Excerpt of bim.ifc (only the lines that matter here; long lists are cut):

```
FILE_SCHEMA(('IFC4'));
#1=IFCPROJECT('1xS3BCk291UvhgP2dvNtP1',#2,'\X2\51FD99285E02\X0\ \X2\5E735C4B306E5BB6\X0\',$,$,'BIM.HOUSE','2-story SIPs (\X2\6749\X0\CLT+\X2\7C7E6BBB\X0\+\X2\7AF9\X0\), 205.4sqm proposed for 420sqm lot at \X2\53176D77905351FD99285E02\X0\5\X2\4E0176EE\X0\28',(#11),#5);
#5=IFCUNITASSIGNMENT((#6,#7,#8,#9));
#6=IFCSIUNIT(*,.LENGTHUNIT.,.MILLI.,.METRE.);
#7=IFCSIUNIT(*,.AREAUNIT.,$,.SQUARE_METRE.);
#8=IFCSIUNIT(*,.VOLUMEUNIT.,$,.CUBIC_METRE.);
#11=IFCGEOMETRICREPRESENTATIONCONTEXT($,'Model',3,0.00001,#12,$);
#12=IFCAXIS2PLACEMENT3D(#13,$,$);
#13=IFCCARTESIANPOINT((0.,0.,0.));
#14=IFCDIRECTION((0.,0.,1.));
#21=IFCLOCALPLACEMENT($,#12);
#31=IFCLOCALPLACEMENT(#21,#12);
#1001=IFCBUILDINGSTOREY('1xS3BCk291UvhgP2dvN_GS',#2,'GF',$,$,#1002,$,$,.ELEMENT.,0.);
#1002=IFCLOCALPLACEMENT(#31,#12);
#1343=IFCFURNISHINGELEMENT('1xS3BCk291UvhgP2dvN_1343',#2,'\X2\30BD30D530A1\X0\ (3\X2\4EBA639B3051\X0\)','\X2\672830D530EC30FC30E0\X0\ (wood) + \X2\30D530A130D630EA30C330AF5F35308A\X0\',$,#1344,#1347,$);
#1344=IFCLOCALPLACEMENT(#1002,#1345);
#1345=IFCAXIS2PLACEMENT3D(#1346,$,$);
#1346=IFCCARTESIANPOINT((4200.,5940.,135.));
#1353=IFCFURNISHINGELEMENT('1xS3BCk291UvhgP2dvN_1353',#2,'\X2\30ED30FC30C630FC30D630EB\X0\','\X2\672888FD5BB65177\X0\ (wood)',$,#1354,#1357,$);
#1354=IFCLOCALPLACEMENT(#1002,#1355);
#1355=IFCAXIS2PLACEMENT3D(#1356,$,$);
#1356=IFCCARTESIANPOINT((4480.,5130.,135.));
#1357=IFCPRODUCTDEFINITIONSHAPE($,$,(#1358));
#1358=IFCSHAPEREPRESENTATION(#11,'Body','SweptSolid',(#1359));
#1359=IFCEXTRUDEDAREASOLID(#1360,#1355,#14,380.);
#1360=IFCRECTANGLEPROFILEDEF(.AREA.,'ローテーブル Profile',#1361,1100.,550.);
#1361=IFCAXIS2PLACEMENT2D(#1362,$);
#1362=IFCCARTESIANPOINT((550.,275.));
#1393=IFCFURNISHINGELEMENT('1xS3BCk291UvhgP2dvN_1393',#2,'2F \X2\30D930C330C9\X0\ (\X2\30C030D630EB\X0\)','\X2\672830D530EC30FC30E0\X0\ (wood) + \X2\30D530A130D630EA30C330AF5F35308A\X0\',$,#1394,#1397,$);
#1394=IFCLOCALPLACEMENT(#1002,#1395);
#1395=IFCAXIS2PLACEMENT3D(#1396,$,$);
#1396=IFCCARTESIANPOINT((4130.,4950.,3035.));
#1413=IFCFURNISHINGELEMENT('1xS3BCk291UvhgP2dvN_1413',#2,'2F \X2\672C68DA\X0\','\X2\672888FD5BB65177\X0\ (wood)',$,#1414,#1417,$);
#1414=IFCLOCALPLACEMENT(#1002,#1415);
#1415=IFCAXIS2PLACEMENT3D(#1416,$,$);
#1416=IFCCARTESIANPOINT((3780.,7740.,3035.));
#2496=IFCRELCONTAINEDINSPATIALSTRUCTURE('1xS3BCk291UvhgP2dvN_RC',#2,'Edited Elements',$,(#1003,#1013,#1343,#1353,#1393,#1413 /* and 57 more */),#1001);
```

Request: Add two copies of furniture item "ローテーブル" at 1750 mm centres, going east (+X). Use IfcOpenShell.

```python
import numpy as np
import ifcopenshell
import ifcopenshell.api.geometry
import ifcopenshell.api.root
import ifcopenshell.util.element
import ifcopenshell.util.placement
import ifcopenshell.util.unit

model = ifcopenshell.open("bim.ifc")
unit_scale = ifcopenshell.util.unit.calculate_unit_scale(model)


def reuse_history(source, copy):
    """copy_class also copies each property set's owner history, people and application; keep the originals."""
    for rel in copy.IsDefinedBy:
        if rel.is_a("IfcRelDefinesByProperties") and (history := rel.RelatingPropertyDefinition.OwnerHistory):
            rel.RelatingPropertyDefinition.OwnerHistory = source.OwnerHistory
            ifcopenshell.util.element.remove_deep2(model, history)


source = model.by_guid("1xS3BCk291UvhgP2dvN_1353")
base = ifcopenshell.util.placement.get_local_placement(source.ObjectPlacement)
step = np.array([1.0, 0.0, 0.0]) * 1.75 / unit_scale

for i in range(1, 3):
    copy = ifcopenshell.api.root.copy_class(model, product=source)
    copy.Representation = ifcopenshell.util.element.copy_deep(
        model, source.Representation, exclude=["IfcGeometricRepresentationContext", "IfcRepresentationMap"]
    )
    reuse_history(source, copy)
    matrix = base.copy()
    matrix[:3, 3] += i * step
    print("added at", matrix[:3, 3].round(3) + 0.0)
    ifcopenshell.api.geometry.edit_object_placement(model, product=copy, matrix=matrix, is_si=False)

model.write("bim-out.ifc")
```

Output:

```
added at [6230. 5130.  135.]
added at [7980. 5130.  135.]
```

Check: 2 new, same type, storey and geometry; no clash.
